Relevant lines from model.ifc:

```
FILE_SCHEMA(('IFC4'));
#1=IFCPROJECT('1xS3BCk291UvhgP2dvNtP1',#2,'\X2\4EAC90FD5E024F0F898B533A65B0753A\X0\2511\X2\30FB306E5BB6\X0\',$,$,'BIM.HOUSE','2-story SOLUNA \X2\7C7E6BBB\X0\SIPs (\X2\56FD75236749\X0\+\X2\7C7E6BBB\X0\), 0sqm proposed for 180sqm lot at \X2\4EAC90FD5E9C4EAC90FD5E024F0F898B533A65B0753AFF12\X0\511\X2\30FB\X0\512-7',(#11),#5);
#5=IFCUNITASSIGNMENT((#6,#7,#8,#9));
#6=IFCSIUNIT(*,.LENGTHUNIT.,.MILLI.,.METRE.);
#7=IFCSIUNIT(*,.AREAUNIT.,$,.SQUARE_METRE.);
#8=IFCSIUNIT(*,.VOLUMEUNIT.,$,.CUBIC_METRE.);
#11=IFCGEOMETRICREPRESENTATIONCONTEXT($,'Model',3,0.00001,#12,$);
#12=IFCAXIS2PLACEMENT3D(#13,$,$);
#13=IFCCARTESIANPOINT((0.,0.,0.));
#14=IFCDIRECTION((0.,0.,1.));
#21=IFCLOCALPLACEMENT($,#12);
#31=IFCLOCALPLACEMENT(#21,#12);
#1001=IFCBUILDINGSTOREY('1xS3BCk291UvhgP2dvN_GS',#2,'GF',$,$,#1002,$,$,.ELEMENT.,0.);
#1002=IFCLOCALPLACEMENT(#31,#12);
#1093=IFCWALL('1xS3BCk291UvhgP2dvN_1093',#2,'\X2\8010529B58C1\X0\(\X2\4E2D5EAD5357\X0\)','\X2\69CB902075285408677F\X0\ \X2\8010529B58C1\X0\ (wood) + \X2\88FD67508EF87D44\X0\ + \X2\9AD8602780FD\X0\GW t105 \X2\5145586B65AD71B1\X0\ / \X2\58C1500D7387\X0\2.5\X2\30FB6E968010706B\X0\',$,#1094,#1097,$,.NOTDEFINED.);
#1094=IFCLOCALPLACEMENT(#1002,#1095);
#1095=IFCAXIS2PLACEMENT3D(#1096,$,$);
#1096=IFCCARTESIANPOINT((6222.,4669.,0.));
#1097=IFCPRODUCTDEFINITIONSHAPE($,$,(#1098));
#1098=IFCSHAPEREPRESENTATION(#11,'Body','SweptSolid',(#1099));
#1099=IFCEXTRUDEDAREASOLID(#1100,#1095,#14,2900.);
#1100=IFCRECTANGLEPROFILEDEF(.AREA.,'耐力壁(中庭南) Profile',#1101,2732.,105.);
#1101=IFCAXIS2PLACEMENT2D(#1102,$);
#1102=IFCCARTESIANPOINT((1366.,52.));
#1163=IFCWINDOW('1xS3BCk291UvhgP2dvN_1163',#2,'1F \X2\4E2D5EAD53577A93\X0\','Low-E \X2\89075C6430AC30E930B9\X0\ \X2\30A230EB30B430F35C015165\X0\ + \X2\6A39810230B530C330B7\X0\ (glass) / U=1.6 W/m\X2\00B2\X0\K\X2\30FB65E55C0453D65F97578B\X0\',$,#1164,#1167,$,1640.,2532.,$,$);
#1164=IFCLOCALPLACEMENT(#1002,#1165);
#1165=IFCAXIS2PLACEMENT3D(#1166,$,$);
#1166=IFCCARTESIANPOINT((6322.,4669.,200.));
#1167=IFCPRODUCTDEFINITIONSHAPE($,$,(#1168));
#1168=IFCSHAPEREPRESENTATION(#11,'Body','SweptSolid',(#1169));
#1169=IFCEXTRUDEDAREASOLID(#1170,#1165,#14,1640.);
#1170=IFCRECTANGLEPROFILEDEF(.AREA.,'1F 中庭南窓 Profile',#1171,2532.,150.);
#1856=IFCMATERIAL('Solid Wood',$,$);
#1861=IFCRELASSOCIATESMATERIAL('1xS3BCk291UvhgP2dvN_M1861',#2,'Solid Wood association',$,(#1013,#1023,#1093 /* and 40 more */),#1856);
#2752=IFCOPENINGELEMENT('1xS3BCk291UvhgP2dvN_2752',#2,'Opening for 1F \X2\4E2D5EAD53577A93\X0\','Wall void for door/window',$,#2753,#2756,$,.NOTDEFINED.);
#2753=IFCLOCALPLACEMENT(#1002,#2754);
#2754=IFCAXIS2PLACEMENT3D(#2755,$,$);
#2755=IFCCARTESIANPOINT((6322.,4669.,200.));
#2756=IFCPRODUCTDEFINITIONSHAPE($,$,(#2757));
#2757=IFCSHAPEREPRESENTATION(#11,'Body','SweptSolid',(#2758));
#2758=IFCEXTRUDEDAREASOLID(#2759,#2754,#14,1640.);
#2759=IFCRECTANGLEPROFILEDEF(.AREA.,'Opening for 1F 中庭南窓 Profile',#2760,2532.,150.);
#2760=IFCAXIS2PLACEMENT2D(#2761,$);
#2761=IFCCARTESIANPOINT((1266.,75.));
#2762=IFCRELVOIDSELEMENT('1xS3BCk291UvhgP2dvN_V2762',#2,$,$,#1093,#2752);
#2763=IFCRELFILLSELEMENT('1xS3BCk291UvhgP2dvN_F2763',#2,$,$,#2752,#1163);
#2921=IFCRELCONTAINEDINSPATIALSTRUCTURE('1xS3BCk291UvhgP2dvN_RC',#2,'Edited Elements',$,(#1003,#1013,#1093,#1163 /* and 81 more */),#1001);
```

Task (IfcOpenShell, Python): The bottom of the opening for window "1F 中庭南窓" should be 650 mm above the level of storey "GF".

```python
import numpy as np
import ifcopenshell
import ifcopenshell.api.geometry
import ifcopenshell.geom
import ifcopenshell.util.element
import ifcopenshell.util.placement
import ifcopenshell.util.shape
import ifcopenshell.util.unit

model = ifcopenshell.open("model.ifc")
unit_scale = ifcopenshell.util.unit.calculate_unit_scale(model)

window = model.by_id(1163)
opening = window.FillsVoids[0].RelatingOpeningElement
storey = ifcopenshell.util.element.get_container(window, ifc_class="IfcBuildingStorey")
level = ifcopenshell.util.placement.get_local_placement(storey.ObjectPlacement)[2, 3]

# The opening's origin need not be at the sill, so measure its lowest point.
shape = ifcopenshell.geom.create_shape(ifcopenshell.geom.settings(), opening)
bottom = ifcopenshell.util.shape.get_shape_bottom_elevation(shape, shape.geometry) / unit_scale
dz = level + 0.65 / unit_scale - bottom

shift = np.array([0.0, 0.0, dz])
# The window is not placed relative to its opening, so move both.
for product in (opening, window):
    matrix = ifcopenshell.util.placement.get_local_placement(product.ObjectPlacement)
    matrix[:3, 3] += shift
    ifcopenshell.api.geometry.edit_object_placement(model, product=product, matrix=matrix, is_si=False)

print(f"moved by {dz * unit_scale:+.3f} m")

model.write("model_rev.ifc")
```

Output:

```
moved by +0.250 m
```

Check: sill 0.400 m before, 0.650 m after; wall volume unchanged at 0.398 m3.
